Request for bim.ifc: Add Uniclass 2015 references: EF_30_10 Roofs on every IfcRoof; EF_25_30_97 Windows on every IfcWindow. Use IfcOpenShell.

First a look at what the model holds.

```python
import ifcopenshell

model = ifcopenshell.open("bim.ifc")
print(model.schema)
print("classifications:", [c.Name for c in model.by_type("IfcClassification")])
for ifc_class in ("IfcDoor", "IfcRoof", "IfcStair", "IfcWall", "IfcWindow"):
    print(ifc_class, len(model.by_type(ifc_class)))
```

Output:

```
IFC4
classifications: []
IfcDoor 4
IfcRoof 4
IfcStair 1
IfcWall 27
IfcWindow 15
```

```python
import ifcopenshell
import ifcopenshell.api.classification

model = ifcopenshell.open("bim.ifc")

system = ifcopenshell.api.classification.add_classification(model, classification="Uniclass 2015")

codes = {
    "IfcRoof": ("EF_30_10", "Roofs"),
    "IfcWindow": ("EF_25_30_97", "Windows"),
}
for ifc_class, (code, name) in codes.items():
    products = model.by_type(ifc_class)
    ifcopenshell.api.classification.add_reference(
        model, products=products, classification=system, identification=code, name=name
    )
    print(code, len(products))

model.write("bim-out.ifc")
```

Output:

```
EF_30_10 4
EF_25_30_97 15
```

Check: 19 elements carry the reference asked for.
